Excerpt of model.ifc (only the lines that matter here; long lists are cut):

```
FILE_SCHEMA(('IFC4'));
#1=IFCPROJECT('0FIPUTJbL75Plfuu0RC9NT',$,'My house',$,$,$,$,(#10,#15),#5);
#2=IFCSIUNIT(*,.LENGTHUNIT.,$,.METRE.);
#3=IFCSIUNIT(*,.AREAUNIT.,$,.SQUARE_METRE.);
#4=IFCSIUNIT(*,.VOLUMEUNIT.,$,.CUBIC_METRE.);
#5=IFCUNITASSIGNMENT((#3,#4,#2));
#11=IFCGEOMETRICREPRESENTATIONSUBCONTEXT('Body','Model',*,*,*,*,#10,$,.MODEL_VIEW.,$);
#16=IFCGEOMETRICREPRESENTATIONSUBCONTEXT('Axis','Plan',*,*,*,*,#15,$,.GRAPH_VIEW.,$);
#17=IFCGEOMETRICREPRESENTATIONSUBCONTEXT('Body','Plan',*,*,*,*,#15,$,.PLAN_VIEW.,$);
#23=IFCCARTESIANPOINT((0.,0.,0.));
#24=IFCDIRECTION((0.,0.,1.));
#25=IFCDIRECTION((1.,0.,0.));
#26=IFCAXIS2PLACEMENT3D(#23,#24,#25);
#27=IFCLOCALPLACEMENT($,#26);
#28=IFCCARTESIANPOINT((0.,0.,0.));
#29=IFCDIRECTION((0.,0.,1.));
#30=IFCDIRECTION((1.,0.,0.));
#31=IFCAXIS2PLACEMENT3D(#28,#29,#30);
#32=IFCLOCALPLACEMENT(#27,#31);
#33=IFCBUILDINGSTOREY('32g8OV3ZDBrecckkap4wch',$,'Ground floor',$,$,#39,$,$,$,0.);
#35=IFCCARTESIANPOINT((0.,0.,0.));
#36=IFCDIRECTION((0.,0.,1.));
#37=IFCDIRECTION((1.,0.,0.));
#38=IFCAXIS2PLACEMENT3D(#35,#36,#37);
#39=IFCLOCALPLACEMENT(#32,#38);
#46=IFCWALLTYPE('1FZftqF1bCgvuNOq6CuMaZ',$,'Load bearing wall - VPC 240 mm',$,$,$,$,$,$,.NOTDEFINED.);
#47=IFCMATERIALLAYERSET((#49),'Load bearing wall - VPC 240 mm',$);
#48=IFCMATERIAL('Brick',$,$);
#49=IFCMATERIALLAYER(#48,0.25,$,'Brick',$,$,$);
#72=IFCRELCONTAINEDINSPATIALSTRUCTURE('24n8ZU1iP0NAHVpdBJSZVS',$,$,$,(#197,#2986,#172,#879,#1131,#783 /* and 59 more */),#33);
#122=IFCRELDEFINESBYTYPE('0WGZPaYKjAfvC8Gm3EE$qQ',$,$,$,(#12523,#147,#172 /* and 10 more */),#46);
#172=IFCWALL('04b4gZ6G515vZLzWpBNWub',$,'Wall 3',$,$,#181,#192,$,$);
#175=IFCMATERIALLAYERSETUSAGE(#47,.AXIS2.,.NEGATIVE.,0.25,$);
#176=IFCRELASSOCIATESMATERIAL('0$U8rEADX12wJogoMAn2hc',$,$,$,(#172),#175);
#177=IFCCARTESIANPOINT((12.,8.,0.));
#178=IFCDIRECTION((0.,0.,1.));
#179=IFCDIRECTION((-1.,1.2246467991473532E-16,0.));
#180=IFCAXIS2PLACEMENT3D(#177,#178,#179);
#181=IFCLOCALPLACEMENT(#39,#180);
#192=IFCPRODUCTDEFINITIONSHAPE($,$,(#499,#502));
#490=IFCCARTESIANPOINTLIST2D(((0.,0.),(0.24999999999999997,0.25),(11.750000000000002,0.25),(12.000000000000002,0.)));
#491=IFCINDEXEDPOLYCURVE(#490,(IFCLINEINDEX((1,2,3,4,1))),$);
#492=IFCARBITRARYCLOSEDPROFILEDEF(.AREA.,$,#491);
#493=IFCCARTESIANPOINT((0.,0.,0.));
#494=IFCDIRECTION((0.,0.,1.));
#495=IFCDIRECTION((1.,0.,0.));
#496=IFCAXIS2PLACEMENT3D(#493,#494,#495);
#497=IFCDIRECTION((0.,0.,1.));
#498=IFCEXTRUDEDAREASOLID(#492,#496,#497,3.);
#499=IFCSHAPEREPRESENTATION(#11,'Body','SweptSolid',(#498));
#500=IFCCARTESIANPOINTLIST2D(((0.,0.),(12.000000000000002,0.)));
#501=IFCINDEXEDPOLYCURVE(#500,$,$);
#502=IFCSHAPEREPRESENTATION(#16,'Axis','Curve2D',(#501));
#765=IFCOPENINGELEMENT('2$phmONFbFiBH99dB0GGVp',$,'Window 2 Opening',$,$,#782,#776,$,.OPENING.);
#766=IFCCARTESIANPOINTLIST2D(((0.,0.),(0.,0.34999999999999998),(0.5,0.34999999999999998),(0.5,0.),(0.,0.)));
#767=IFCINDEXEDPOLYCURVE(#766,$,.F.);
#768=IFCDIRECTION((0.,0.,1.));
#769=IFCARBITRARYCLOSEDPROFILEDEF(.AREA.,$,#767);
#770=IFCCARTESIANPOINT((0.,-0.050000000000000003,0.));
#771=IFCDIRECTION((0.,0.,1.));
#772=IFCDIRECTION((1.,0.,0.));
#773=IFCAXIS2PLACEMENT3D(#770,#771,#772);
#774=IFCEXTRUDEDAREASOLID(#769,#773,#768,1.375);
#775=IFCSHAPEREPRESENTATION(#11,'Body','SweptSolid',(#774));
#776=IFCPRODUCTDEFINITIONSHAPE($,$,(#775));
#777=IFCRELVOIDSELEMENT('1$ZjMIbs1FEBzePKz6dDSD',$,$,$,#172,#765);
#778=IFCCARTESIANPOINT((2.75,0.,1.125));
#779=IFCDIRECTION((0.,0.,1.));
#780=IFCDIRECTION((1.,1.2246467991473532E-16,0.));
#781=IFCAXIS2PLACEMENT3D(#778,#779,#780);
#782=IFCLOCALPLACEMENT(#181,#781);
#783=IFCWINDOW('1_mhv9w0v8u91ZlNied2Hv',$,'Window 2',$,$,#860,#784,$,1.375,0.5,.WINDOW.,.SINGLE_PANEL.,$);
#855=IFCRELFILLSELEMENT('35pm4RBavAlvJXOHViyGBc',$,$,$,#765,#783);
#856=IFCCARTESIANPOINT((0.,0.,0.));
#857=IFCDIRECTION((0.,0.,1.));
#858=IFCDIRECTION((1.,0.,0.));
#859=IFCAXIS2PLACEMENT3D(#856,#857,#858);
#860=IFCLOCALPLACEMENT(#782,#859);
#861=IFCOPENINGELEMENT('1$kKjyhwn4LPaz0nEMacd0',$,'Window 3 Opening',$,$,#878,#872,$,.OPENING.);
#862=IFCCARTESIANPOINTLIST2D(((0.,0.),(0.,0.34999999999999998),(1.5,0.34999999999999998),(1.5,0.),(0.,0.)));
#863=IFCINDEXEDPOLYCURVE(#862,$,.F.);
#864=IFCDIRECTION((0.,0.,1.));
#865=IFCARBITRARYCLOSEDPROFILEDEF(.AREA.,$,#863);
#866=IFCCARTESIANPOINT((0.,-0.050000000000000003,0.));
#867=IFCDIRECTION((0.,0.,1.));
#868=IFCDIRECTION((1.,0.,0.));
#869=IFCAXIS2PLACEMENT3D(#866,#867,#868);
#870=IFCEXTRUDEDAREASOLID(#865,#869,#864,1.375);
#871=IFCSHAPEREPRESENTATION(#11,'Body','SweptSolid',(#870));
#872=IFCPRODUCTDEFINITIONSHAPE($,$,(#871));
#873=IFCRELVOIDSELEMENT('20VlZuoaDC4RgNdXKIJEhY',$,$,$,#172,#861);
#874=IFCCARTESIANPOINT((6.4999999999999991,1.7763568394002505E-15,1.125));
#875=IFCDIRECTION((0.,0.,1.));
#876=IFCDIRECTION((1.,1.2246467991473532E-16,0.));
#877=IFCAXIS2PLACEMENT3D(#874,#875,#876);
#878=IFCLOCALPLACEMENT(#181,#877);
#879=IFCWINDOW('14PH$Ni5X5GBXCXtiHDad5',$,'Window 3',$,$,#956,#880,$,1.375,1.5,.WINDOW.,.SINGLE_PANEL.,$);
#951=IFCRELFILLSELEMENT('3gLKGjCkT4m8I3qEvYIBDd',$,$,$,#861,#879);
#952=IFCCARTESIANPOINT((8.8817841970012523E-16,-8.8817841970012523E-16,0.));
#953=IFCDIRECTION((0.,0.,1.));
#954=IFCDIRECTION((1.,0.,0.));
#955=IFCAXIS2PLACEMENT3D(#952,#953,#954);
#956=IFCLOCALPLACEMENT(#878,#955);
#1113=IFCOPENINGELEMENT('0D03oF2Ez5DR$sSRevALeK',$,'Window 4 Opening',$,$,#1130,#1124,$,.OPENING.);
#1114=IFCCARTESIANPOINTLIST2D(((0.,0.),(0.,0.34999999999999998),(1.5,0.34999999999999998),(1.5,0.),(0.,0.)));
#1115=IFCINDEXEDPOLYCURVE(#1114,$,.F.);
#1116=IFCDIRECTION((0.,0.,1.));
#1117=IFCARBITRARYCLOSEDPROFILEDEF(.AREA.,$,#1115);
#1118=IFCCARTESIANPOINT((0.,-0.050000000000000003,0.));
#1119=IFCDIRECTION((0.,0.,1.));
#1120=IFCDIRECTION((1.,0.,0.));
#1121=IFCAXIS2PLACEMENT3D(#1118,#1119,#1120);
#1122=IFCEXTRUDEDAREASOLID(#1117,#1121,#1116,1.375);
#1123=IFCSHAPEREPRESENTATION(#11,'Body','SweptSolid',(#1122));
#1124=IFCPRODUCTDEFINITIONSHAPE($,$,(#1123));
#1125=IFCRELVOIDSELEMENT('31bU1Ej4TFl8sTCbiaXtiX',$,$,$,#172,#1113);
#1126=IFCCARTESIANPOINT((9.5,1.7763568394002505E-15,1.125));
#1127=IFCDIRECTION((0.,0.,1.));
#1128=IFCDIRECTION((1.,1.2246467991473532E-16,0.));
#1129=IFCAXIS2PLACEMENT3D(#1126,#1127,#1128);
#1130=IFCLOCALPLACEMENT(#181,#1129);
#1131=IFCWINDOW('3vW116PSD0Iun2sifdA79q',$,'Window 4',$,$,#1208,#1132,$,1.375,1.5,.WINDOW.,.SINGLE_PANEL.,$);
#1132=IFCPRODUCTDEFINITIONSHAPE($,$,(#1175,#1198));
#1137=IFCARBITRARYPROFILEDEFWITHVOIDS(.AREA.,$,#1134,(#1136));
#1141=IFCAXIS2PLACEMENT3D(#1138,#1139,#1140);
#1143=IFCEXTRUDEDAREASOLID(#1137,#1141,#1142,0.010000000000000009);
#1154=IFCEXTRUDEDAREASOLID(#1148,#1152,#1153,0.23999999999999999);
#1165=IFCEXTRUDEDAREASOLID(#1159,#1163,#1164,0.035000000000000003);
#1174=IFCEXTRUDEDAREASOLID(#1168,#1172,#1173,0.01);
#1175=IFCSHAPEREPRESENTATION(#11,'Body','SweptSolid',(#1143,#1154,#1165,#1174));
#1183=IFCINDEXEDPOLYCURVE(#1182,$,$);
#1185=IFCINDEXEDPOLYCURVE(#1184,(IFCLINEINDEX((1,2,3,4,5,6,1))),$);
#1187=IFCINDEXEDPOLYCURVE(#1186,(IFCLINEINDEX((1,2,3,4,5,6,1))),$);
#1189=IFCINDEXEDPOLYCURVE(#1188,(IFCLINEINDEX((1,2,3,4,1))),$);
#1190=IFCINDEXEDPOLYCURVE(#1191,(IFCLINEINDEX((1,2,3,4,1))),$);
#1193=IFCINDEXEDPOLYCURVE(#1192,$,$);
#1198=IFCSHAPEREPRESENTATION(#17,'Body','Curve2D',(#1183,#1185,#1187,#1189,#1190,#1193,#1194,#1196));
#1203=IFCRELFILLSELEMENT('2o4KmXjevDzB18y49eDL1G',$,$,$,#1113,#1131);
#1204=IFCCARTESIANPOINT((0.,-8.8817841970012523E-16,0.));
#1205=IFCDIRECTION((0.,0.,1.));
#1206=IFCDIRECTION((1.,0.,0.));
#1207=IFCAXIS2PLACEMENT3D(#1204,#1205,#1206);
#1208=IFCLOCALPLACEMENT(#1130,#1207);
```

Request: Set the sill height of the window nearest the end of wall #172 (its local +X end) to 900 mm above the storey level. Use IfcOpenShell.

```python
import numpy as np
import ifcopenshell
import ifcopenshell.api.geometry
import ifcopenshell.geom
import ifcopenshell.util.element
import ifcopenshell.util.placement
import ifcopenshell.util.shape
import ifcopenshell.util.unit

model = ifcopenshell.open("model.ifc")
unit_scale = ifcopenshell.util.unit.calculate_unit_scale(model)

window = model.by_guid("3vW116PSD0Iun2sifdA79q")
opening = window.FillsVoids[0].RelatingOpeningElement
storey = ifcopenshell.util.element.get_container(window, ifc_class="IfcBuildingStorey")
level = ifcopenshell.util.placement.get_local_placement(storey.ObjectPlacement)[2, 3]

# The opening's origin need not be at the sill, so measure its lowest point.
shape = ifcopenshell.geom.create_shape(ifcopenshell.geom.settings(), opening)
bottom = ifcopenshell.util.shape.get_shape_bottom_elevation(shape, shape.geometry) / unit_scale
dz = level + 0.9 / unit_scale - bottom

shift = np.array([0.0, 0.0, dz])
# The window is placed relative to its opening, so it follows when the opening moves.
matrix = ifcopenshell.util.placement.get_local_placement(opening.ObjectPlacement)
matrix[:3, 3] += shift
ifcopenshell.api.geometry.edit_object_placement(
    model, product=opening, matrix=matrix, is_si=False, should_transform_children=True
)

print(f"moved by {dz * unit_scale:+.3f} m")

model.write("model_v2.ifc")
```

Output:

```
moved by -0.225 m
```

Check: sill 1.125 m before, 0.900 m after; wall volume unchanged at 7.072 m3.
